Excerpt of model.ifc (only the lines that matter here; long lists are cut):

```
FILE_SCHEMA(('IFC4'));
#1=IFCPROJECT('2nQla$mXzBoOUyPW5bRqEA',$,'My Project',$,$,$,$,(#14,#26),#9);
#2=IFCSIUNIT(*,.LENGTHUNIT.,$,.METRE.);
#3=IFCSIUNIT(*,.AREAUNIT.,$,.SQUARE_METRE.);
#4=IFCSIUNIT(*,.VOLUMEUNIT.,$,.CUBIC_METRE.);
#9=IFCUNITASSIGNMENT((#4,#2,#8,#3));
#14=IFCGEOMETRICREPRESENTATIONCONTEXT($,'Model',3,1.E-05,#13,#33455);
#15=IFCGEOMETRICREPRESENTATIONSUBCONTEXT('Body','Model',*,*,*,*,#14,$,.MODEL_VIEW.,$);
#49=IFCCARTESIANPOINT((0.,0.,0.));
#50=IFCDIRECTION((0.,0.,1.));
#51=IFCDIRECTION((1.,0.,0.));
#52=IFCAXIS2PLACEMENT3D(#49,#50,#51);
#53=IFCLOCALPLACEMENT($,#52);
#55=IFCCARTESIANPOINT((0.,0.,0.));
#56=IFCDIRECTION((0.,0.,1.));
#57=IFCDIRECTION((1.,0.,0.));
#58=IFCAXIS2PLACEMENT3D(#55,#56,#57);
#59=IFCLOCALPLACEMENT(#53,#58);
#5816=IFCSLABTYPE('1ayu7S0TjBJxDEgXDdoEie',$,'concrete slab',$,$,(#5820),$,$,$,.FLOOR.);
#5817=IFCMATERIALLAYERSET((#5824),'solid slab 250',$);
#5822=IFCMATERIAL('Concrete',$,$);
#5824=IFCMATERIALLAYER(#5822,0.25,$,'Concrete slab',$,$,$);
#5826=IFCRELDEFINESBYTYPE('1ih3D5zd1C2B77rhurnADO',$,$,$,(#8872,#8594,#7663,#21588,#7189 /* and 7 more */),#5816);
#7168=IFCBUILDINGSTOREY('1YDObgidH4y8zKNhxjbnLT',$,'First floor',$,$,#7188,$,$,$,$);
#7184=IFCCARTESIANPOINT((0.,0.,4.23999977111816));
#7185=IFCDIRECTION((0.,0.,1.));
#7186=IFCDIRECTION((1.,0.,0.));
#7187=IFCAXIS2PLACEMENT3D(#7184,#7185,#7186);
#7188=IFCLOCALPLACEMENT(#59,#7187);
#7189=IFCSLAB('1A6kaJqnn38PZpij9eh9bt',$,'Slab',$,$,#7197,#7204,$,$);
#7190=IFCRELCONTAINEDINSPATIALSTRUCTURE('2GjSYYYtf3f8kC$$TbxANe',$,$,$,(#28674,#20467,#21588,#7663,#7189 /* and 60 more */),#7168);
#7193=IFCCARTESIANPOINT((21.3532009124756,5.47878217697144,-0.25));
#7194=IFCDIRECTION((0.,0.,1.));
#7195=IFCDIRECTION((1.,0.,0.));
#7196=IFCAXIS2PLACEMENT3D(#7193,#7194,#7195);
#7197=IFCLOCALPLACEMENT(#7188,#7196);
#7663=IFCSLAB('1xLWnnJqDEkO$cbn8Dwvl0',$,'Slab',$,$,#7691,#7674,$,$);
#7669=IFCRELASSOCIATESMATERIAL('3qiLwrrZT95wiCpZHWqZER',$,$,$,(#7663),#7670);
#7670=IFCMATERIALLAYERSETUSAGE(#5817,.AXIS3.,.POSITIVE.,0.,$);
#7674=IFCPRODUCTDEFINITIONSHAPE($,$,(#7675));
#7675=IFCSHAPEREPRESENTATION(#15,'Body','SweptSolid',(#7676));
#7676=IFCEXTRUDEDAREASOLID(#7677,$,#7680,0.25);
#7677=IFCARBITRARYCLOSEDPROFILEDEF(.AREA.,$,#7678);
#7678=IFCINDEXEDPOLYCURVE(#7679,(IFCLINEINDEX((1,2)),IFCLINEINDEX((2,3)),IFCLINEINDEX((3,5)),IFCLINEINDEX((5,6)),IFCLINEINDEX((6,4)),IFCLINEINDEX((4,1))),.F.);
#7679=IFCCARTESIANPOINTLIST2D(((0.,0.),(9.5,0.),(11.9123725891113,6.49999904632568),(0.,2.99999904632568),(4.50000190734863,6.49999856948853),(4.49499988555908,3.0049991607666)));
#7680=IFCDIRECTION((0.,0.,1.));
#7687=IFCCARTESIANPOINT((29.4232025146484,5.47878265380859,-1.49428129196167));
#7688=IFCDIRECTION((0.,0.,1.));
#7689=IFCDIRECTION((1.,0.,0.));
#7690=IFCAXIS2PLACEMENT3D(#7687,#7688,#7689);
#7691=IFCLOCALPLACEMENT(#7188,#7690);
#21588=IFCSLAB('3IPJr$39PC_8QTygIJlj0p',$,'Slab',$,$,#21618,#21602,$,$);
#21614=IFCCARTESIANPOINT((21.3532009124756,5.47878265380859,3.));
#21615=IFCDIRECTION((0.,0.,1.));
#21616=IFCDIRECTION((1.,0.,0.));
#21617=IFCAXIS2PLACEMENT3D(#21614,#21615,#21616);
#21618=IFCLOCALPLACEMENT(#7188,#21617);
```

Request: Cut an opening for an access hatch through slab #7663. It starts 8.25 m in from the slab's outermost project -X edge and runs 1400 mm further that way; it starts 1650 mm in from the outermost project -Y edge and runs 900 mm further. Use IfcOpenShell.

```python
import numpy as np
import ifcopenshell
import ifcopenshell.api.feature
import ifcopenshell.api.geometry
import ifcopenshell.api.root
import ifcopenshell.geom
import ifcopenshell.util.placement
import ifcopenshell.util.representation
import ifcopenshell.util.shape
import ifcopenshell.util.unit

model = ifcopenshell.open("model.ifc")
unit_scale = ifcopenshell.util.unit.calculate_unit_scale(model)
settings = ifcopenshell.geom.settings()


def volume(element):
    """Net volume in cubic metres, openings subtracted."""
    shape = ifcopenshell.geom.create_shape(settings, element)
    return ifcopenshell.util.shape.get_volume(shape.geometry)


slab = model.by_id(7663)
before = volume(slab)

# Extent in the slab's own axes, in metres. The edges named are its -X and -Y sides.
slab_shape = ifcopenshell.geom.create_shape(settings, slab)
vertices = ifcopenshell.util.shape.get_vertices(slab_shape.geometry)
x_min, y_min, bottom = vertices.min(axis=0)
top = vertices[:, 2].max()

opening = ifcopenshell.api.root.create_entity(model, ifc_class="IfcOpeningElement", name="Access hatch opening", predefined_type="OPENING")
context = ifcopenshell.util.representation.get_context(model, "Model", "Body", "MODEL_VIEW")
width, depth = 1.4, 0.9
outline = [(0.0, 0.0), (width, 0.0), (width, depth), (0.0, depth), (0.0, 0.0)]
# Overshoot both faces by 50 mm so the cut is clean.
shape = ifcopenshell.api.geometry.add_slab_representation(
    model, context=context, depth=top - bottom + 0.1, polyline=outline
)
ifcopenshell.api.geometry.assign_representation(model, product=opening, representation=shape)

matrix = ifcopenshell.util.placement.get_local_placement(slab.ObjectPlacement)
matrix[:, 3] = matrix @ np.append(np.array([x_min + 8.25, y_min + 1.65, bottom - 0.05]) / unit_scale, 1.0)
ifcopenshell.api.geometry.edit_object_placement(model, product=opening, matrix=matrix, is_si=False)
ifcopenshell.api.feature.add_feature(model, feature=opening, element=slab)

after = volume(slab)

print(f"slab volume {before:.3f} -> {after:.3f} m3")

model.write("model_rev.ifc")
```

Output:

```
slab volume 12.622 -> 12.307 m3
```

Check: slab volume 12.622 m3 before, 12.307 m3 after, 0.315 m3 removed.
